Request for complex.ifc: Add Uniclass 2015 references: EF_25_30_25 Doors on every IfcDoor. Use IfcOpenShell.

First a look at what the model holds.

```python
import ifcopenshell

model = ifcopenshell.open("complex.ifc")
print(model.schema)
print("classifications:", [c.Name for c in model.by_type("IfcClassification")])
for ifc_class in ("IfcDoor", "IfcRoof", "IfcStair", "IfcWall", "IfcWindow"):
    print(ifc_class, len(model.by_type(ifc_class)))
```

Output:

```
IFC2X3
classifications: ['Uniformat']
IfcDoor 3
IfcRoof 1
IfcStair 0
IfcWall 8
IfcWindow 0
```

```python
import ifcopenshell
import ifcopenshell.api.classification

model = ifcopenshell.open("complex.ifc")

# IFC2X3 requires Source and Edition and has no link from the project to the system.
system = model.create_entity("IfcClassification", Source="NBS", Edition="2015", Name="Uniclass 2015")

codes = {
    "IfcDoor": ("EF_25_30_25", "Doors"),
}
for ifc_class, (code, name) in codes.items():
    products = model.by_type(ifc_class)
    ifcopenshell.api.classification.add_reference(
        model, products=products, classification=system, identification=code, name=name
    )
    print(code, len(products))

model.write("complex_rev.ifc")
```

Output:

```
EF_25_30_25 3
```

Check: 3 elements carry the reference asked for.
